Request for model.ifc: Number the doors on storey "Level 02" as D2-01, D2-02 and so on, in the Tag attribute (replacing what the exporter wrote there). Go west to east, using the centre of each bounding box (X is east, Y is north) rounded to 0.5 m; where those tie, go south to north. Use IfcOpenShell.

First a look at what the model holds.

```python
import ifcopenshell
import ifcopenshell.util.element
import ifcopenshell.util.placement

model = ifcopenshell.open("model.ifc")
print(model.schema)
storey = next(s for s in model.by_type("IfcBuildingStorey") if s.Name == "Level 02")
doors = [e for e in ifcopenshell.util.element.get_decomposition(storey) if e.is_a("IfcDoor")]
for e in sorted(doors, key=lambda e: e.id()):
    origin = ifcopenshell.util.placement.get_local_placement(e.ObjectPlacement)[:3, 3]
    print(e.id(), e.Tag, e.Name, origin.round(2) + 0.0, sep=" | ")
```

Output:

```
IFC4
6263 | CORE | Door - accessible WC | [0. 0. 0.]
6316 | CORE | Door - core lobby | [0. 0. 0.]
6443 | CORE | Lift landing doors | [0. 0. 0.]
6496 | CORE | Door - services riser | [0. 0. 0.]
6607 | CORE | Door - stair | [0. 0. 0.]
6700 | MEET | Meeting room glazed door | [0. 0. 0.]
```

```python
import ifcopenshell
import ifcopenshell.geom
import ifcopenshell.util.element
import ifcopenshell.util.shape

model = ifcopenshell.open("model.ifc")
settings = ifcopenshell.geom.settings()
settings.set("use-world-coords", True)


def centre(element):
    shape = ifcopenshell.geom.create_shape(settings, element)
    return ifcopenshell.util.shape.get_bbox_centroid(shape.geometry)


storey = next(s for s in model.by_type("IfcBuildingStorey") if s.Name == "Level 02")
doors = [e for e in ifcopenshell.util.element.get_decomposition(storey) if e.is_a("IfcDoor")]

# Insertion points can sit at a corner or the storey origin, so sort by the geometry (in metres).
centres = {e: centre(e) for e in doors}
doors.sort(key=lambda e: (round(centres[e][0] / 0.5), centres[e][1]))

for i, e in enumerate(doors, start=1):
    number = f"D2-{i:02d}"
    e.Tag = number
    print(e.id(), number)

model.write("model_v2.ifc")
```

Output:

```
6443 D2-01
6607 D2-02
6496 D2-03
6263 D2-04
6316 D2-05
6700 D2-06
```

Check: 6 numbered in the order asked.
